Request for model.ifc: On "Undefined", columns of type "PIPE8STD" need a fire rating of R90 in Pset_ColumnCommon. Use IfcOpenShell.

First a look at what the model holds.

```python
import ifcopenshell
import ifcopenshell.util.element

model = ifcopenshell.open("model.ifc")
print(model.schema)
storey = next(s for s in model.by_type("IfcBuildingStorey") if s.Name == "Undefined")
columns = [e for e in ifcopenshell.util.element.get_decomposition(storey) if e.is_a("IfcColumn")]
seen = {}
for e in columns:
    element_type = ifcopenshell.util.element.get_type(e)
    key = (element_type.Name if element_type != e and element_type else None, ifcopenshell.util.element.get_pset(e, "Pset_ColumnCommon", "FireRating"))
    seen[key] = seen.get(key, 0) + 1
for (name, value), count in sorted(seen.items(), key=str):
    print(count, "x", name, "|", value)
```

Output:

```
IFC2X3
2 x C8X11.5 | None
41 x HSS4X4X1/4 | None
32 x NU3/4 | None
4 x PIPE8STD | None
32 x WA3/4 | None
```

```python
import ifcopenshell
import ifcopenshell.api.pset
import ifcopenshell.util.element

model = ifcopenshell.open("model.ifc")

storey = next(s for s in model.by_type("IfcBuildingStorey") if s.Name == "Undefined")
columns = [e for e in ifcopenshell.util.element.get_decomposition(storey) if e.is_a("IfcColumn")]

count = 0
for e in columns:
    element_type = ifcopenshell.util.element.get_type(e)
    if element_type in (None, e) or element_type.Name != "PIPE8STD":
        continue
    found = ifcopenshell.util.element.get_pset(e, "Pset_ColumnCommon", should_inherit=False)
    if found:
        pset = model.by_id(found["id"])
        if len(ifcopenshell.util.element.get_elements_by_pset(pset)) > 1:
            pset = ifcopenshell.api.pset.unshare_pset(model, products=[e], pset=pset)[0]
    else:
        pset = ifcopenshell.api.pset.add_pset(model, product=e, name="Pset_ColumnCommon")
    ifcopenshell.api.pset.edit_pset(model, pset=pset, properties={"FireRating": "R90"})
    count += 1

print(count, "columns updated")

model.write("model_updated.ifc")
```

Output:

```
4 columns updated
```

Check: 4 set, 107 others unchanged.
